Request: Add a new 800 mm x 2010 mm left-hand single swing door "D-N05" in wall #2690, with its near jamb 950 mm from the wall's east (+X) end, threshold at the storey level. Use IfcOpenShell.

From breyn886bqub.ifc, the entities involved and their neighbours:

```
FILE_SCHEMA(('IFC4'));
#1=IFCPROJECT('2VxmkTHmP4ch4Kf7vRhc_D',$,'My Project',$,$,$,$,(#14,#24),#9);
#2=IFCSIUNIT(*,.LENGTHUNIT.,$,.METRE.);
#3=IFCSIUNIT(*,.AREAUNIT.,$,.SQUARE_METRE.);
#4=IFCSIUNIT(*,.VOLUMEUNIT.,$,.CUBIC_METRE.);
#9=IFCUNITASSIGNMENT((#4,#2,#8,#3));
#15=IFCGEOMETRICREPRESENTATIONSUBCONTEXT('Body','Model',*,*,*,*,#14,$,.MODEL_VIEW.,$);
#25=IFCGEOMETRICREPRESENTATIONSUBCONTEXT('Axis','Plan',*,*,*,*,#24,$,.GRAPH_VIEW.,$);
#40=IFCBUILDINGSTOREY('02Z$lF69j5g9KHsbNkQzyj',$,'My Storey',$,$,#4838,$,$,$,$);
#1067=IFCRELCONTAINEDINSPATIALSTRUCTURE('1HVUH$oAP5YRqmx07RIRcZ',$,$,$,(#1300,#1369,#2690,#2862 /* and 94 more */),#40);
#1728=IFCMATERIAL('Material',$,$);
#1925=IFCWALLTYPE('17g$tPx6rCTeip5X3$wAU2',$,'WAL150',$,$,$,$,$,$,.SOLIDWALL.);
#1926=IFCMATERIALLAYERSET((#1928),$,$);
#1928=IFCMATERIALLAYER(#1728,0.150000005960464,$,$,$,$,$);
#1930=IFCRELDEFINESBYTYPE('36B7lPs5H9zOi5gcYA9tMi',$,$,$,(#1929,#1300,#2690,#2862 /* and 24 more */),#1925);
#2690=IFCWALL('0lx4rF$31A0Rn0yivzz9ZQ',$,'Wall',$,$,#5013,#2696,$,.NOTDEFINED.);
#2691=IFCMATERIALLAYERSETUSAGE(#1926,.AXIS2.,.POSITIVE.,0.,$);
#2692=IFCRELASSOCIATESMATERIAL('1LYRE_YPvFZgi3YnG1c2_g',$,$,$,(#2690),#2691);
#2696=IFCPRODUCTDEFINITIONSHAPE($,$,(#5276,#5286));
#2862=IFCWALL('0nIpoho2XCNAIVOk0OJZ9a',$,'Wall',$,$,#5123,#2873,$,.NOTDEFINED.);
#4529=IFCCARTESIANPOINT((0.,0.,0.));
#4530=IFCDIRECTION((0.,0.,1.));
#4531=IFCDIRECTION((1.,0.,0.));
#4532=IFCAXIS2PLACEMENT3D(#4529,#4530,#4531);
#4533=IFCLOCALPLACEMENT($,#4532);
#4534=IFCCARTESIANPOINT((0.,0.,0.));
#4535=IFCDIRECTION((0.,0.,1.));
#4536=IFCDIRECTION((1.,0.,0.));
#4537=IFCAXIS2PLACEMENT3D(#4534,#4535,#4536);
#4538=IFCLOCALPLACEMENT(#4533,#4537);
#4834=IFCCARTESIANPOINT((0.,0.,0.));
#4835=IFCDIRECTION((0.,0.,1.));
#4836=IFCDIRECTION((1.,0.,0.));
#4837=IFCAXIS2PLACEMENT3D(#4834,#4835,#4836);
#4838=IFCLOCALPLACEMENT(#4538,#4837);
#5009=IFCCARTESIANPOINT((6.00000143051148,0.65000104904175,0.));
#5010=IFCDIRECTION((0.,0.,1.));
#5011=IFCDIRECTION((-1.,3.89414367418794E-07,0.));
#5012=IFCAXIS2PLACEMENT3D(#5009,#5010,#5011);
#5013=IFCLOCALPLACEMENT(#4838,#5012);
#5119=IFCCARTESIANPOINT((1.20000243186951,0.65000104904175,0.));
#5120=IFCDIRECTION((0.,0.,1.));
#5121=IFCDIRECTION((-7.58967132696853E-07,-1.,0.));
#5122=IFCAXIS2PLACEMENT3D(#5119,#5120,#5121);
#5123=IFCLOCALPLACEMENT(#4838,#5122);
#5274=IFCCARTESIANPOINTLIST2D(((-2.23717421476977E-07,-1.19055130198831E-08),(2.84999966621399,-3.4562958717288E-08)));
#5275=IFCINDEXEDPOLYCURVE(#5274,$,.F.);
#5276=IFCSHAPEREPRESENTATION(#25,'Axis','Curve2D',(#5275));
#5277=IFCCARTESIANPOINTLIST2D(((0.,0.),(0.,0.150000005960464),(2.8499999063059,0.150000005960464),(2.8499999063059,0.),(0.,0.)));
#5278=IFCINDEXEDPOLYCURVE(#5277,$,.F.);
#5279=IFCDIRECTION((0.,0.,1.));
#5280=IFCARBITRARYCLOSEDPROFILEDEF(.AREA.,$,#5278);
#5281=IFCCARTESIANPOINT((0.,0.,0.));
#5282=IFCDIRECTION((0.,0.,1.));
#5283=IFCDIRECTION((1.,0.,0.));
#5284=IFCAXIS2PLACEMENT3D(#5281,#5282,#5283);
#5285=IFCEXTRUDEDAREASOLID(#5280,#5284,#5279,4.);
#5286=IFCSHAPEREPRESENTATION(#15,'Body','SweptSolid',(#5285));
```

```python
import numpy as np
import ifcopenshell
import ifcopenshell.api.feature
import ifcopenshell.api.geometry
import ifcopenshell.api.root
import ifcopenshell.api.spatial
import ifcopenshell.geom
import ifcopenshell.util.element
import ifcopenshell.util.placement
import ifcopenshell.util.representation
import ifcopenshell.util.shape
import ifcopenshell.util.unit

model = ifcopenshell.open("breyn886bqub.ifc")
unit_scale = ifcopenshell.util.unit.calculate_unit_scale(model)
settings = ifcopenshell.geom.settings()


def volume(element):
    """Net volume in cubic metres, openings subtracted."""
    shape = ifcopenshell.geom.create_shape(settings, element)
    return ifcopenshell.util.shape.get_volume(shape.geometry)


wall = model.by_guid("0lx4rF$31A0Rn0yivzz9ZQ")
storey = ifcopenshell.util.element.get_container(wall, ifc_class="IfcBuildingStorey")
context = ifcopenshell.util.representation.get_context(model, "Model", "Body", "MODEL_VIEW")
before = volume(wall)

width, height, from_end, sill = 0.8, 2.01, 0.95, 0.0  # metres

# The wall runs along its own X axis, and the end named is its -X end.
wall_shape = ifcopenshell.geom.create_shape(settings, wall)
x, y, z = ifcopenshell.util.shape.get_vertices(wall_shape.geometry).T
start = x.min() + from_end
face, thickness = float(y.min()), float(y.max() - y.min())
wall_matrix = ifcopenshell.util.placement.get_local_placement(wall.ObjectPlacement)
level = ifcopenshell.util.placement.get_local_placement(storey.ObjectPlacement)[2, 3]


def in_wall(x, y):
    """Placement at x, y metres in the wall's axes, at sill height."""
    matrix = wall_matrix.copy()
    matrix[:, 3] = wall_matrix @ np.array([x / unit_scale, y / unit_scale, 0.0, 1.0])
    matrix[2, 3] = level + sill / unit_scale
    return matrix


# Opening: a box that overshoots both wall faces by 50 mm.
opening = ifcopenshell.api.root.create_entity(model, ifc_class="IfcOpeningElement", predefined_type="OPENING")
box = ifcopenshell.api.geometry.add_wall_representation(
    model, context=context, length=width, height=height, thickness=thickness + 0.1
)
ifcopenshell.api.geometry.assign_representation(model, product=opening, representation=box)
ifcopenshell.api.geometry.edit_object_placement(model, product=opening, matrix=in_wall(start, face - 0.05), is_si=False)
ifcopenshell.api.feature.add_feature(model, feature=opening, element=wall)

door = ifcopenshell.api.root.create_entity(model, ifc_class="IfcDoor", name="D-N05", predefined_type="DOOR")
door.OverallWidth, door.OverallHeight = width / unit_scale, height / unit_scale
door.OperationType = "SINGLE_SWING_LEFT"
body = ifcopenshell.api.geometry.add_door_representation(
    model,
    context=context,
    overall_width=door.OverallWidth,
    overall_height=door.OverallHeight,
    operation_type="SINGLE_SWING_LEFT",
    lining_properties={"LiningDepth": thickness / unit_scale, "ThresholdDepth": thickness / unit_scale},
)
ifcopenshell.api.geometry.assign_representation(model, product=door, representation=body)
ifcopenshell.api.spatial.assign_container(model, products=[door], relating_structure=storey)
ifcopenshell.api.feature.add_filling(model, opening=opening, element=door)

# The lining spans the wall, so the door starts at the wall face.
ifcopenshell.api.geometry.edit_object_placement(model, product=door, matrix=in_wall(start, face), is_si=False)

after = volume(wall)

print(f"wall volume {before:.3f} -> {after:.3f} m3")

model.write("breyn886bqub_edited.ifc")
```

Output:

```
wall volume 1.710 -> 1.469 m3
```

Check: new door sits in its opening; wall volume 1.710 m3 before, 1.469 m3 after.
